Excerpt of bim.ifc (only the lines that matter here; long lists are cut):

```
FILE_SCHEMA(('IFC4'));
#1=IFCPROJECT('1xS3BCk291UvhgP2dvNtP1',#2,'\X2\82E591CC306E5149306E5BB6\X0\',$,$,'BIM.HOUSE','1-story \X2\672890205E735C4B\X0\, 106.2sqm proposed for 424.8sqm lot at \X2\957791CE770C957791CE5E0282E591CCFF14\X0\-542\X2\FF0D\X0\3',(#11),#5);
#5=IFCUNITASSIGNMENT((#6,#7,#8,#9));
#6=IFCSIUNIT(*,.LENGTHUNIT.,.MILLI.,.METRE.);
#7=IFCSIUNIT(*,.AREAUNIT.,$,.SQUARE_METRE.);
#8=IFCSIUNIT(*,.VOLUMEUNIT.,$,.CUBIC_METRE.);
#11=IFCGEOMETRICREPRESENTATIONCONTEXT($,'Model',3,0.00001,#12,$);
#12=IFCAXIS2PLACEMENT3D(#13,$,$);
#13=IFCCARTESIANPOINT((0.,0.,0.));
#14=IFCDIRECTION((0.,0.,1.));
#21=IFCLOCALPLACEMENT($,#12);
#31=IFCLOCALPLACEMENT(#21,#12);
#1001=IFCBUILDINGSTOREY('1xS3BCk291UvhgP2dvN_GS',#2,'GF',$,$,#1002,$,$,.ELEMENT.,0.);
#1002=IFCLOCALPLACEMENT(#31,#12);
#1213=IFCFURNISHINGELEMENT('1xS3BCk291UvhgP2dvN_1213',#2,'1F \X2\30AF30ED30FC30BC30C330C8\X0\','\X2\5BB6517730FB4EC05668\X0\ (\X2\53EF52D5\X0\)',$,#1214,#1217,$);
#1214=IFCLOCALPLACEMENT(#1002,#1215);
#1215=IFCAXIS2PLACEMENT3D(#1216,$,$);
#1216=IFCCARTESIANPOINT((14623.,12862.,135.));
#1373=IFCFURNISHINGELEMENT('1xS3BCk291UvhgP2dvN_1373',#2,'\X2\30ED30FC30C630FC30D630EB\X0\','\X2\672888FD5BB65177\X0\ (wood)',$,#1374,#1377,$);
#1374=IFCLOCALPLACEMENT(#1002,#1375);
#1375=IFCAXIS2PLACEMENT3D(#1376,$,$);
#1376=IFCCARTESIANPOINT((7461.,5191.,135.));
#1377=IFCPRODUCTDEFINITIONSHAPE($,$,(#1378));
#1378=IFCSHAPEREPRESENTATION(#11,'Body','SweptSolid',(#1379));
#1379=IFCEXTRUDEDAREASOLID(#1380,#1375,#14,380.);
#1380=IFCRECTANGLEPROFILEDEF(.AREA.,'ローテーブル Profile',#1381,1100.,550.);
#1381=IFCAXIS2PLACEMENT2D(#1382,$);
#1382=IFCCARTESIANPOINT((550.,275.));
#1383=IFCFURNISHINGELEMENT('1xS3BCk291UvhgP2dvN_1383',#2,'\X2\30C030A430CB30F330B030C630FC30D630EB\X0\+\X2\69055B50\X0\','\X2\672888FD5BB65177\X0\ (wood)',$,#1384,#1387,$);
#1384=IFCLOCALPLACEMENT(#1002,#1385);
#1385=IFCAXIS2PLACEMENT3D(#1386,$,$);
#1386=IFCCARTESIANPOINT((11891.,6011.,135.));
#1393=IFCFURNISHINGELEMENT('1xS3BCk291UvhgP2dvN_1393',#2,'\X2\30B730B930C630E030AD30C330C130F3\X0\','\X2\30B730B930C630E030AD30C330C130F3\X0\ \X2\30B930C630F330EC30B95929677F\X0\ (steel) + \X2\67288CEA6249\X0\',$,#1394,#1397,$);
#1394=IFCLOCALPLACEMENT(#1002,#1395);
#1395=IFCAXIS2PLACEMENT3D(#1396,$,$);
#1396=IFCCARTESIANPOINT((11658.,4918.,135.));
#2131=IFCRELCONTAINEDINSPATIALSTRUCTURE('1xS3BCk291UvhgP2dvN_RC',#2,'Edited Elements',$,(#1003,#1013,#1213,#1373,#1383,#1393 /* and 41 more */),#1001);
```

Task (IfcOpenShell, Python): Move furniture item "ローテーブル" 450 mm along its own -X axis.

```python
import ifcopenshell
import ifcopenshell.api.geometry
import ifcopenshell.util.placement
import ifcopenshell.util.unit

model = ifcopenshell.open("bim.ifc")
unit_scale = ifcopenshell.util.unit.calculate_unit_scale(model)

item = model.by_id(1373)
matrix = ifcopenshell.util.placement.get_local_placement(item.ObjectPlacement)
matrix[:3, 3] -= matrix[:3, 0] * 0.45 / unit_scale
ifcopenshell.api.geometry.edit_object_placement(model, product=item, matrix=matrix, is_si=False)

print(ifcopenshell.util.placement.get_local_placement(item.ObjectPlacement).round(3) + 0.0)

model.write("bim_v2.ifc")
```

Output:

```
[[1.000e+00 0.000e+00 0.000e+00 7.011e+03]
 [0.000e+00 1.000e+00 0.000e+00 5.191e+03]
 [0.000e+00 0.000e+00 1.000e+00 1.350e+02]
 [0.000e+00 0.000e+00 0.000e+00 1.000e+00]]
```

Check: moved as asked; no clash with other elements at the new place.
